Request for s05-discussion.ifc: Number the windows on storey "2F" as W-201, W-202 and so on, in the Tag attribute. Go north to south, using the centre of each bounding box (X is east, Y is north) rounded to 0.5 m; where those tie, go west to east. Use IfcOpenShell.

First a look at what the model holds.

```python
import ifcopenshell
import ifcopenshell.util.element
import ifcopenshell.util.placement

model = ifcopenshell.open("s05-discussion.ifc")
print(model.schema)
storey = next(s for s in model.by_type("IfcBuildingStorey") if s.Name == "2F")
windows = [e for e in ifcopenshell.util.element.get_decomposition(storey) if e.is_a("IfcWindow")]
for e in sorted(windows, key=lambda e: e.id()):
    origin = ifcopenshell.util.placement.get_local_placement(e.ObjectPlacement)[:3, 3]
    print(e.id(), e.Tag, e.Name, origin.round(2) + 0.0, sep=" | ")
```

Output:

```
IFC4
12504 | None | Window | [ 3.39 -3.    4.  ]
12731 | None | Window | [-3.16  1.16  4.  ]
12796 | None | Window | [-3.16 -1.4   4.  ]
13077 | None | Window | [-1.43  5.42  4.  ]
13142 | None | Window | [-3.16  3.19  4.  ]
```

```python
import ifcopenshell
import ifcopenshell.geom
import ifcopenshell.util.element
import ifcopenshell.util.shape

model = ifcopenshell.open("s05-discussion.ifc")
settings = ifcopenshell.geom.settings()
settings.set("use-world-coords", True)


def centre(element):
    shape = ifcopenshell.geom.create_shape(settings, element)
    return ifcopenshell.util.shape.get_bbox_centroid(shape.geometry)


storey = next(s for s in model.by_type("IfcBuildingStorey") if s.Name == "2F")
windows = [e for e in ifcopenshell.util.element.get_decomposition(storey) if e.is_a("IfcWindow")]

# Insertion points can sit at a corner or the storey origin, so sort by the geometry (in metres).
centres = {e: centre(e) for e in windows}
windows.sort(key=lambda e: (-round(centres[e][1] / 0.5), centres[e][0]))

for i, e in enumerate(windows, start=1):
    number = f"W-2{i:02d}"
    e.Tag = number
    print(e.id(), number)

model.write("s05-discussion_edited.ifc")
```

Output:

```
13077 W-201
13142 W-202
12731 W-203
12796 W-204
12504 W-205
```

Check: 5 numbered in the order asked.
